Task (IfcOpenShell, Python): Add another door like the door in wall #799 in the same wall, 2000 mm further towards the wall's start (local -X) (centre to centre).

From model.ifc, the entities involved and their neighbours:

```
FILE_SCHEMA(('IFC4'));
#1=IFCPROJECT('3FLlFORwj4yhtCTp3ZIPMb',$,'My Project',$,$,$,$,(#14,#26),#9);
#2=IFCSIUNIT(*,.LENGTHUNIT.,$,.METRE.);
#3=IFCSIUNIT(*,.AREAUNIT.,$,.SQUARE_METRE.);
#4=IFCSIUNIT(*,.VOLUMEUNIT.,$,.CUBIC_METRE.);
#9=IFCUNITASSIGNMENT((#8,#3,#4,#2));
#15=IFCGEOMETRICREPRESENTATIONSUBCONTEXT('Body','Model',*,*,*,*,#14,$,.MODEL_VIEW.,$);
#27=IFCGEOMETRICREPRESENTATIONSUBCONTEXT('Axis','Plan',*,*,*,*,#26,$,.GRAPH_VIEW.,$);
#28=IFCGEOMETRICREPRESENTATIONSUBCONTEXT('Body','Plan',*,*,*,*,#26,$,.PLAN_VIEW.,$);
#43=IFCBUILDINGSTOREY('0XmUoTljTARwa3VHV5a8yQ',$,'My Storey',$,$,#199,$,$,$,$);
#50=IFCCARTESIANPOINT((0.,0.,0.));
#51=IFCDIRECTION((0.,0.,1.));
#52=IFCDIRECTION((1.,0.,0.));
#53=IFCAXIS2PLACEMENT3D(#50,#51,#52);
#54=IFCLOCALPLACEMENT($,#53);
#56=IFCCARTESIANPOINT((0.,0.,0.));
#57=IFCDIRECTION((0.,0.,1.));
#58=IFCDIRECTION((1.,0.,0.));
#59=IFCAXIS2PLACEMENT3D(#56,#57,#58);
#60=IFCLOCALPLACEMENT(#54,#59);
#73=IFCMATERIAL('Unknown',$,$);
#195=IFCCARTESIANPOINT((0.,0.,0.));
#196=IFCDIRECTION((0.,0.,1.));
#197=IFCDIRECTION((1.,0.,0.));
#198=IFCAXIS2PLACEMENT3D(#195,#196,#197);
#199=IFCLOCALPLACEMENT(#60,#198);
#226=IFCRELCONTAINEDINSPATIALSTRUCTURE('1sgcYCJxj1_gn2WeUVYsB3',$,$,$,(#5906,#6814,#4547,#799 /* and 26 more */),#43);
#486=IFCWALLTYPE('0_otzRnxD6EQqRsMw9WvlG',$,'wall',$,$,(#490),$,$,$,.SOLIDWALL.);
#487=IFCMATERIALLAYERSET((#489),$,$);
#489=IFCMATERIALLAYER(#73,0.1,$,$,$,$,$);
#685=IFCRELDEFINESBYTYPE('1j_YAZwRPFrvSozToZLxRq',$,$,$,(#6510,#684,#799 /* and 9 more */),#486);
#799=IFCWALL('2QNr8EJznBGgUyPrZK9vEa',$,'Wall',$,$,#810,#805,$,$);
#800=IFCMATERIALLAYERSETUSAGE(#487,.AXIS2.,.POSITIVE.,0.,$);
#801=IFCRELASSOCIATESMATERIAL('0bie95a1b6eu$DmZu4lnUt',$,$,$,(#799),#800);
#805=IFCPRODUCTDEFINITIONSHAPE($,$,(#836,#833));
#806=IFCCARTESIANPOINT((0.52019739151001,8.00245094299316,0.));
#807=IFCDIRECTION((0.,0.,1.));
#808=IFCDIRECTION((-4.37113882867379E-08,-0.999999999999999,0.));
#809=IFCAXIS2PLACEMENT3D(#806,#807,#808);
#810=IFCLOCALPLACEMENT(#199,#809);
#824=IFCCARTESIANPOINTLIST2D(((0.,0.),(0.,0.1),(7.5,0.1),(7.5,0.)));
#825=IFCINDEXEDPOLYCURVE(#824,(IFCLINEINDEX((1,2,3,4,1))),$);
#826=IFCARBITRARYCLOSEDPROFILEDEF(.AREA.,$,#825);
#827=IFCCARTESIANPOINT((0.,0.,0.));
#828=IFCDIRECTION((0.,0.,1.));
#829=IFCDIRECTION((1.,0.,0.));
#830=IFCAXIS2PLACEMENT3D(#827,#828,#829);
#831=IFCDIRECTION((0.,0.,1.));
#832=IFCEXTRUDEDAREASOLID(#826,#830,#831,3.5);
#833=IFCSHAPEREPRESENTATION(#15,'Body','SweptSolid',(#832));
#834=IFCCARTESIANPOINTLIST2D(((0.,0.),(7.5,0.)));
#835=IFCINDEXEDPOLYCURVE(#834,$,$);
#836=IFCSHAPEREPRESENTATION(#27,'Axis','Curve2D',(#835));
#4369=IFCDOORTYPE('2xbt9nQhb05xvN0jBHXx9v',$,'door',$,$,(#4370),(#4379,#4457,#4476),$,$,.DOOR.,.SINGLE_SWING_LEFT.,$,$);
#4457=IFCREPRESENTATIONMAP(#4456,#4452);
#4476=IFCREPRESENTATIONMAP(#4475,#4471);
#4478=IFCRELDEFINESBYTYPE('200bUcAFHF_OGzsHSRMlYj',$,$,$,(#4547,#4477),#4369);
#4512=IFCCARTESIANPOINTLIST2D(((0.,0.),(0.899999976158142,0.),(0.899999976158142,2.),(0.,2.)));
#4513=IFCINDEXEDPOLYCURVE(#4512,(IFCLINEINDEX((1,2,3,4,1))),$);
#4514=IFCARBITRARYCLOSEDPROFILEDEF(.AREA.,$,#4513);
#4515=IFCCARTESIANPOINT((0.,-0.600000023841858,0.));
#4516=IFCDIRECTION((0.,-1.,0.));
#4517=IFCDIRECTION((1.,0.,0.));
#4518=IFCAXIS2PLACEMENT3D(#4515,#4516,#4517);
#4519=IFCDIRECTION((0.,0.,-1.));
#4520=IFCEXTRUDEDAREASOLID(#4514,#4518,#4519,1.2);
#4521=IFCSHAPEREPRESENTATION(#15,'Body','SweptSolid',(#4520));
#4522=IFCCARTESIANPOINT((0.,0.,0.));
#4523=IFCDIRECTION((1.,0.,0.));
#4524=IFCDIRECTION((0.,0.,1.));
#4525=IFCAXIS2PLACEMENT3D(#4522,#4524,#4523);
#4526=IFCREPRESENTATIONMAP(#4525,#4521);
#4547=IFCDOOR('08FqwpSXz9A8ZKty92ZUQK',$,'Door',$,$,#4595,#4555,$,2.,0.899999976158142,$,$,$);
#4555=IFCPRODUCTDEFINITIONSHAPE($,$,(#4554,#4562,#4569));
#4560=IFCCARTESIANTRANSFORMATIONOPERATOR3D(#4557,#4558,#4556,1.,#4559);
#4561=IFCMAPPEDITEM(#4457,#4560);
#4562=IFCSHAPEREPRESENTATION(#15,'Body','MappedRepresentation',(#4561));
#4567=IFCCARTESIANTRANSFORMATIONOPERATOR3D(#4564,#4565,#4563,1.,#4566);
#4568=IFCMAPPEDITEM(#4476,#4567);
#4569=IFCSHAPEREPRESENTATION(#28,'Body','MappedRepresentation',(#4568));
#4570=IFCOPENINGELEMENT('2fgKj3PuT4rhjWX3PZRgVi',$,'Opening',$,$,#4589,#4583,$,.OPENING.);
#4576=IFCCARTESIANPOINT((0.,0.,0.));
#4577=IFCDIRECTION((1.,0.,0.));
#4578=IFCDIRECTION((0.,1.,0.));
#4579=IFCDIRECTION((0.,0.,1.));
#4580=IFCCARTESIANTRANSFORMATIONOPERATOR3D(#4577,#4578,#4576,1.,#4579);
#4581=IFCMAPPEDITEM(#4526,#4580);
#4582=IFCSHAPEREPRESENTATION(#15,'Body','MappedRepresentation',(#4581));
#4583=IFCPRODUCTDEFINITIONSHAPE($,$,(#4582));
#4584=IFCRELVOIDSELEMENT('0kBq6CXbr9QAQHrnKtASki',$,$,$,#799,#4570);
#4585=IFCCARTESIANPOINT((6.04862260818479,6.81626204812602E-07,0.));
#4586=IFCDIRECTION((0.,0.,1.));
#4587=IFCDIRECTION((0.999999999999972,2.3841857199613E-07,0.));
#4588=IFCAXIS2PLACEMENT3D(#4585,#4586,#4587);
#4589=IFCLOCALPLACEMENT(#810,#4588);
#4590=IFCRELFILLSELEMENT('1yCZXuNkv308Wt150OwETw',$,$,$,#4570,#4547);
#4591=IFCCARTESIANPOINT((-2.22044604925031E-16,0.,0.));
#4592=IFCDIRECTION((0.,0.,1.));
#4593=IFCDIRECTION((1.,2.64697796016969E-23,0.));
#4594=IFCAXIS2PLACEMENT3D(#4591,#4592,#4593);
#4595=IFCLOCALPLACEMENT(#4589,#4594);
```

```python
import ifcopenshell
import ifcopenshell.api.feature
import ifcopenshell.api.geometry
import ifcopenshell.api.root
import ifcopenshell.geom
import ifcopenshell.util.element
import ifcopenshell.util.placement
import ifcopenshell.util.shape

model = ifcopenshell.open("model.ifc")
settings = ifcopenshell.geom.settings()


def volume(element):
    """Net volume in cubic metres, openings subtracted."""
    shape = ifcopenshell.geom.create_shape(settings, element)
    return ifcopenshell.util.shape.get_volume(shape.geometry)


door = model.by_id(4547)
opening = door.FillsVoids[0].RelatingOpeningElement
wall = opening.VoidsElements[0].RelatingBuildingElement
before = volume(wall)
shift = ifcopenshell.util.placement.get_local_placement(wall.ObjectPlacement)[:3, 0] * -2.0

# copy_class copies the void relationship, type, container and properties, but no geometry.
new_opening = ifcopenshell.api.root.copy_class(model, product=opening)
new_opening.Representation = ifcopenshell.util.element.copy_deep(
    model, opening.Representation, exclude=["IfcGeometricRepresentationContext", "IfcRepresentationMap"]
)
new_door = ifcopenshell.api.root.copy_class(model, product=door)
new_door.Representation = ifcopenshell.util.element.copy_deep(
    model, door.Representation, exclude=["IfcGeometricRepresentationContext", "IfcRepresentationMap"]
)
ifcopenshell.api.feature.add_filling(model, opening=new_opening, element=new_door)

for old, new in ((opening, new_opening), (door, new_door)):
    matrix = ifcopenshell.util.placement.get_local_placement(old.ObjectPlacement)
    matrix[:3, 3] += shift
    ifcopenshell.api.geometry.edit_object_placement(model, product=new, matrix=matrix, is_si=False)

after = volume(wall)

print(f"wall volume {before:.3f} -> {after:.3f} m3")

model.write("model_edited.ifc")
```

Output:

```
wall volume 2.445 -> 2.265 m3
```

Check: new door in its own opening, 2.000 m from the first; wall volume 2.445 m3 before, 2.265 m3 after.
